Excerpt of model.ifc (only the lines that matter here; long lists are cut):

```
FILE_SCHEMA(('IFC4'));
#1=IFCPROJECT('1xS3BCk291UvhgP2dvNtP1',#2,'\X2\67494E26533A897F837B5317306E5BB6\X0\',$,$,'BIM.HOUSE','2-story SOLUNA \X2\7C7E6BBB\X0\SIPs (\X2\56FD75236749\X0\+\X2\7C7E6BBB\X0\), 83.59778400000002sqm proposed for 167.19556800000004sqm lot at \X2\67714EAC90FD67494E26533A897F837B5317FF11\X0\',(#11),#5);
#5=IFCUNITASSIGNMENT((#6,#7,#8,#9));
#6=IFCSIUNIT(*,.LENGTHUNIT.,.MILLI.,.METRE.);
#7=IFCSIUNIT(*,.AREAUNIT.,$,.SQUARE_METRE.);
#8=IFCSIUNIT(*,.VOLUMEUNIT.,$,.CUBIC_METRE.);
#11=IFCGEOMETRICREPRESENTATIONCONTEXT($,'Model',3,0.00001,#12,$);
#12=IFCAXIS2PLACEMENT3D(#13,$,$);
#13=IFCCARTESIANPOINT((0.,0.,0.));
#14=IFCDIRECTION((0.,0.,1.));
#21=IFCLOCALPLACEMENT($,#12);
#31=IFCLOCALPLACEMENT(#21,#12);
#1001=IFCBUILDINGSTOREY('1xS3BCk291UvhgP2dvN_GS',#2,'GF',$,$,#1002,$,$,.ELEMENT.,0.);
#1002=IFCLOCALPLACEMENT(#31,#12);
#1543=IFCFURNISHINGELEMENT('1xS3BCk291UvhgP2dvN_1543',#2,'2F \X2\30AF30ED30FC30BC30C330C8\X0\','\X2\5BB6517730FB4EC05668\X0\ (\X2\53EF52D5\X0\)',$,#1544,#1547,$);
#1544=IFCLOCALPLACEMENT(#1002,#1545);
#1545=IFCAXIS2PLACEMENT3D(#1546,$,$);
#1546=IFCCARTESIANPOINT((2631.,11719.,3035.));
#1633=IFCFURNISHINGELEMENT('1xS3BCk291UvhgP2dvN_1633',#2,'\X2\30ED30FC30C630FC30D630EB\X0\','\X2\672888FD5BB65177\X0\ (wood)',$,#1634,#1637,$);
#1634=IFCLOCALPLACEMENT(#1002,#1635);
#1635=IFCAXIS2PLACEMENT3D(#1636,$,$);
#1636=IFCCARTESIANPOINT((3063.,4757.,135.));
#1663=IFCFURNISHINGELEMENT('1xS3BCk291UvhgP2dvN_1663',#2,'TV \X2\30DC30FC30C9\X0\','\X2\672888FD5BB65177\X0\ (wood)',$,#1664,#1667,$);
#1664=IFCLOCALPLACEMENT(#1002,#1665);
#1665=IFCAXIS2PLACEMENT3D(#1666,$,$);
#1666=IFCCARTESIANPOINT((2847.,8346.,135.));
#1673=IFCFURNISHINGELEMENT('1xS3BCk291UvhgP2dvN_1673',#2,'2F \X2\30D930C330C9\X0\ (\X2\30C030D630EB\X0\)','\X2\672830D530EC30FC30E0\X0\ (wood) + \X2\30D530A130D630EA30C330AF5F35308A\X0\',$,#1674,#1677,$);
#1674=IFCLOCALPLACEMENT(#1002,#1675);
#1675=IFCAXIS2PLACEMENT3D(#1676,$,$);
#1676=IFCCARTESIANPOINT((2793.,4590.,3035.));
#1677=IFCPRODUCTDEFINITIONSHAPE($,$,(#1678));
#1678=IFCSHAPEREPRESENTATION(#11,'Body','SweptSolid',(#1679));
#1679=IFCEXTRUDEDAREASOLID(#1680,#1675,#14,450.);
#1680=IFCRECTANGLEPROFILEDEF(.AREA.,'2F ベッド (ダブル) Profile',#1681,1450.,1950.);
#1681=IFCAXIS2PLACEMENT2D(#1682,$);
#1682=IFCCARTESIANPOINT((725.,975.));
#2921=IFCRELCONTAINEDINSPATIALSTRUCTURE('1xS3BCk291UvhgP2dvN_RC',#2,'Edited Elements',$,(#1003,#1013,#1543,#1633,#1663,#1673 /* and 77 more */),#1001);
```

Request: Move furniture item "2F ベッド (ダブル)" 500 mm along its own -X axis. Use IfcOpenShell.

```python
import ifcopenshell
import ifcopenshell.api.geometry
import ifcopenshell.util.placement

model = ifcopenshell.open("model.ifc")

item = model.by_guid("1xS3BCk291UvhgP2dvN_1673")
matrix = ifcopenshell.util.placement.get_local_placement(item.ObjectPlacement)
matrix[:3, 3] -= matrix[:3, 0] * 500.0
ifcopenshell.api.geometry.edit_object_placement(model, product=item, matrix=matrix, is_si=False)

print(ifcopenshell.util.placement.get_local_placement(item.ObjectPlacement).round(3) + 0.0)

model.write("model_edited.ifc")
```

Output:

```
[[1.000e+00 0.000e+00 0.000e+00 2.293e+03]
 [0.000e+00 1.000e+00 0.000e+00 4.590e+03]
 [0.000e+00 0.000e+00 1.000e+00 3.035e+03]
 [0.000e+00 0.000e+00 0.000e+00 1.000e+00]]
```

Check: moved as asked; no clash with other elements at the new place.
